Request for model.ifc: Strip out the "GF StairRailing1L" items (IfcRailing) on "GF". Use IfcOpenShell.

First a look at what the model holds.

```python
import ifcopenshell
import ifcopenshell.util.element

model = ifcopenshell.open("model.ifc")
print(model.schema)
storey = next(s for s in model.by_type("IfcBuildingStorey") if s.Name == "GF")
railings = [e for e in ifcopenshell.util.element.get_decomposition(storey) if e.is_a("IfcRailing")]
seen = {}
for e in railings:
    element_type = ifcopenshell.util.element.get_type(e)
    name = element_type.Name if element_type not in (None, e) else None
    seen[name] = seen.get(name, 0) + 1
for name, count in sorted(seen.items(), key=str):
    print(count, "x", name)
```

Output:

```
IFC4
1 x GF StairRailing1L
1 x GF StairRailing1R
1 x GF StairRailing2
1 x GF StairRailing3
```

```python
import ifcopenshell
import ifcopenshell.api.root
import ifcopenshell.util.element

model = ifcopenshell.open("model.ifc")

storey = next(s for s in model.by_type("IfcBuildingStorey") if s.Name == "GF")
railings = [e for e in ifcopenshell.util.element.get_decomposition(storey) if e.is_a("IfcRailing")]
targets = [e for e in railings if (t := ifcopenshell.util.element.get_type(e)) not in (None, e) and t.Name == "GF StairRailing1L"]

for e in targets:
    ifcopenshell.api.root.remove_product(model, product=e)
print(len(targets), "removed")

model.write("model_updated.ifc")
```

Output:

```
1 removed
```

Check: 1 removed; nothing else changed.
